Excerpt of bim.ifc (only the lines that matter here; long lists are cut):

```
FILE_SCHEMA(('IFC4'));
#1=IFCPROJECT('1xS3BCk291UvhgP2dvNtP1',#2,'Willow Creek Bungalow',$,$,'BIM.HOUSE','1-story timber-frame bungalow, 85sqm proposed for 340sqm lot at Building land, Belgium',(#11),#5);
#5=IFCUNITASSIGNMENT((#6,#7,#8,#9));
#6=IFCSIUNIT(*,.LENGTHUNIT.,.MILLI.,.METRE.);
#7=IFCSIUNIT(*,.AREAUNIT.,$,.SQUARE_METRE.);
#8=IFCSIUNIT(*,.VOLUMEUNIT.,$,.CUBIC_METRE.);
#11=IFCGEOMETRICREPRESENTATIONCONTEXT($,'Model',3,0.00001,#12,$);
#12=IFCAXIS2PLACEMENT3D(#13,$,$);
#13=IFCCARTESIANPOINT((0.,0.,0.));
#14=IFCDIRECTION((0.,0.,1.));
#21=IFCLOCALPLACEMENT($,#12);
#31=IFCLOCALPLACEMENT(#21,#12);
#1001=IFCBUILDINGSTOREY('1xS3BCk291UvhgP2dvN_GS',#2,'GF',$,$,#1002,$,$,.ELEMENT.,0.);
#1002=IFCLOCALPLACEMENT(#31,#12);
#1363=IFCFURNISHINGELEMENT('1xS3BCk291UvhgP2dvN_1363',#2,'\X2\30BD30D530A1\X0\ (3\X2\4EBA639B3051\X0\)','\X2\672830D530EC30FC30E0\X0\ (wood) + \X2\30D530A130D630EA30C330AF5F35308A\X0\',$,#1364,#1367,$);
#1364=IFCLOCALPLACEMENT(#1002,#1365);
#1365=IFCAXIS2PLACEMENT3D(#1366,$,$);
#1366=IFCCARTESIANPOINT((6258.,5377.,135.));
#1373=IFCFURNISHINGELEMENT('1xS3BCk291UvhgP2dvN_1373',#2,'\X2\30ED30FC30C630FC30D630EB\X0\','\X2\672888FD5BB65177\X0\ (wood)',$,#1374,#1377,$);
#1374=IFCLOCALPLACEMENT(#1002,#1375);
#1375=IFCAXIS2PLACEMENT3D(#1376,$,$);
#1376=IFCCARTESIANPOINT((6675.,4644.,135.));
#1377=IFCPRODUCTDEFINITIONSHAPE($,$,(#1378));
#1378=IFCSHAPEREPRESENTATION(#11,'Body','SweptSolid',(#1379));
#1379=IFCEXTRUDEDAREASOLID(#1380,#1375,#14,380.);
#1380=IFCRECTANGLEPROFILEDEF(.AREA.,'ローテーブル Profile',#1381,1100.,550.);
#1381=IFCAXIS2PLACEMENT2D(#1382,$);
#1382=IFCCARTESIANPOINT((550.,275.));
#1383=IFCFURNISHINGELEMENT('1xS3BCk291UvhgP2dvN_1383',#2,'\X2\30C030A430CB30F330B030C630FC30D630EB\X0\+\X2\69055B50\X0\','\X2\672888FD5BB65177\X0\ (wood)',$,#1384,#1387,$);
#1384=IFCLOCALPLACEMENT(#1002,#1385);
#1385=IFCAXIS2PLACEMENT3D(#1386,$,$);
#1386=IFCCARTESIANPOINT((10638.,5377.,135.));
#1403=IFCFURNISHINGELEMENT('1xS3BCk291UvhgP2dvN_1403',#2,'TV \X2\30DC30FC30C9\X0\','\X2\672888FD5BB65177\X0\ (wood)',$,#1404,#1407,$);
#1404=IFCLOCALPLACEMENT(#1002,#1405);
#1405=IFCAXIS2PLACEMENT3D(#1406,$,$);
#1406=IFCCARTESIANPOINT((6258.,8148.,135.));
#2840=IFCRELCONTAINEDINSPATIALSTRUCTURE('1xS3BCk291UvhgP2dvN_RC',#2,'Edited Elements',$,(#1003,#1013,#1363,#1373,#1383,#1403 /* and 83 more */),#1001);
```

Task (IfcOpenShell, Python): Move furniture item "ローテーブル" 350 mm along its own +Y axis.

```python
import ifcopenshell
import ifcopenshell.api.geometry
import ifcopenshell.util.placement
import ifcopenshell.util.unit

model = ifcopenshell.open("bim.ifc")
unit_scale = ifcopenshell.util.unit.calculate_unit_scale(model)

item = model.by_guid("1xS3BCk291UvhgP2dvN_1373")
matrix = ifcopenshell.util.placement.get_local_placement(item.ObjectPlacement)
matrix[:3, 3] += matrix[:3, 1] * 0.35 / unit_scale
ifcopenshell.api.geometry.edit_object_placement(model, product=item, matrix=matrix, is_si=False)

print(ifcopenshell.util.placement.get_local_placement(item.ObjectPlacement).round(3) + 0.0)

model.write("bim-out.ifc")
```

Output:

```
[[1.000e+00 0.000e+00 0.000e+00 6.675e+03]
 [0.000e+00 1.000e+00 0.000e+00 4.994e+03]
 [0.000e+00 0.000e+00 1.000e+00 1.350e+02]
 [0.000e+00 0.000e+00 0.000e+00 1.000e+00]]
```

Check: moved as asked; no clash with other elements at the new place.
